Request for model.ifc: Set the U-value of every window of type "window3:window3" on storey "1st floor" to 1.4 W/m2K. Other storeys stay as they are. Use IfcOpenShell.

First a look at what the model holds.

```python
import ifcopenshell
import ifcopenshell.util.element

model = ifcopenshell.open("model.ifc")
print(model.schema)
storey = next(s for s in model.by_type("IfcBuildingStorey") if s.Name == "1st floor")
windows = [e for e in ifcopenshell.util.element.get_decomposition(storey) if e.is_a("IfcWindow")]
seen = {}
for e in windows:
    element_type = ifcopenshell.util.element.get_type(e)
    key = (element_type.Name if element_type != e and element_type else None, ifcopenshell.util.element.get_pset(e, "Pset_WindowCommon", "ThermalTransmittance"))
    seen[key] = seen.get(key, 0) + 1
for (name, value), count in sorted(seen.items(), key=str):
    print(count, "x", name, "|", value)
```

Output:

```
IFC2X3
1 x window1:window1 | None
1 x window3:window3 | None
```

```python
import ifcopenshell
import ifcopenshell.api.pset
import ifcopenshell.util.element

model = ifcopenshell.open("model.ifc")

storey = next(s for s in model.by_type("IfcBuildingStorey") if s.Name == "1st floor")
windows = [e for e in ifcopenshell.util.element.get_decomposition(storey) if e.is_a("IfcWindow")]

count = 0
for e in windows:
    element_type = ifcopenshell.util.element.get_type(e)
    if element_type in (None, e) or element_type.Name != "window3:window3":
        continue
    # add_pset returns the element's existing set when there is one.
    pset = ifcopenshell.api.pset.add_pset(model, product=e, name="Pset_WindowCommon")
    ifcopenshell.api.pset.edit_pset(model, pset=pset, properties={"ThermalTransmittance": 1.4})
    count += 1

print(count, "windows updated")

model.write("model-out.ifc")
```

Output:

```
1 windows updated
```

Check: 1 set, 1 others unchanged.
